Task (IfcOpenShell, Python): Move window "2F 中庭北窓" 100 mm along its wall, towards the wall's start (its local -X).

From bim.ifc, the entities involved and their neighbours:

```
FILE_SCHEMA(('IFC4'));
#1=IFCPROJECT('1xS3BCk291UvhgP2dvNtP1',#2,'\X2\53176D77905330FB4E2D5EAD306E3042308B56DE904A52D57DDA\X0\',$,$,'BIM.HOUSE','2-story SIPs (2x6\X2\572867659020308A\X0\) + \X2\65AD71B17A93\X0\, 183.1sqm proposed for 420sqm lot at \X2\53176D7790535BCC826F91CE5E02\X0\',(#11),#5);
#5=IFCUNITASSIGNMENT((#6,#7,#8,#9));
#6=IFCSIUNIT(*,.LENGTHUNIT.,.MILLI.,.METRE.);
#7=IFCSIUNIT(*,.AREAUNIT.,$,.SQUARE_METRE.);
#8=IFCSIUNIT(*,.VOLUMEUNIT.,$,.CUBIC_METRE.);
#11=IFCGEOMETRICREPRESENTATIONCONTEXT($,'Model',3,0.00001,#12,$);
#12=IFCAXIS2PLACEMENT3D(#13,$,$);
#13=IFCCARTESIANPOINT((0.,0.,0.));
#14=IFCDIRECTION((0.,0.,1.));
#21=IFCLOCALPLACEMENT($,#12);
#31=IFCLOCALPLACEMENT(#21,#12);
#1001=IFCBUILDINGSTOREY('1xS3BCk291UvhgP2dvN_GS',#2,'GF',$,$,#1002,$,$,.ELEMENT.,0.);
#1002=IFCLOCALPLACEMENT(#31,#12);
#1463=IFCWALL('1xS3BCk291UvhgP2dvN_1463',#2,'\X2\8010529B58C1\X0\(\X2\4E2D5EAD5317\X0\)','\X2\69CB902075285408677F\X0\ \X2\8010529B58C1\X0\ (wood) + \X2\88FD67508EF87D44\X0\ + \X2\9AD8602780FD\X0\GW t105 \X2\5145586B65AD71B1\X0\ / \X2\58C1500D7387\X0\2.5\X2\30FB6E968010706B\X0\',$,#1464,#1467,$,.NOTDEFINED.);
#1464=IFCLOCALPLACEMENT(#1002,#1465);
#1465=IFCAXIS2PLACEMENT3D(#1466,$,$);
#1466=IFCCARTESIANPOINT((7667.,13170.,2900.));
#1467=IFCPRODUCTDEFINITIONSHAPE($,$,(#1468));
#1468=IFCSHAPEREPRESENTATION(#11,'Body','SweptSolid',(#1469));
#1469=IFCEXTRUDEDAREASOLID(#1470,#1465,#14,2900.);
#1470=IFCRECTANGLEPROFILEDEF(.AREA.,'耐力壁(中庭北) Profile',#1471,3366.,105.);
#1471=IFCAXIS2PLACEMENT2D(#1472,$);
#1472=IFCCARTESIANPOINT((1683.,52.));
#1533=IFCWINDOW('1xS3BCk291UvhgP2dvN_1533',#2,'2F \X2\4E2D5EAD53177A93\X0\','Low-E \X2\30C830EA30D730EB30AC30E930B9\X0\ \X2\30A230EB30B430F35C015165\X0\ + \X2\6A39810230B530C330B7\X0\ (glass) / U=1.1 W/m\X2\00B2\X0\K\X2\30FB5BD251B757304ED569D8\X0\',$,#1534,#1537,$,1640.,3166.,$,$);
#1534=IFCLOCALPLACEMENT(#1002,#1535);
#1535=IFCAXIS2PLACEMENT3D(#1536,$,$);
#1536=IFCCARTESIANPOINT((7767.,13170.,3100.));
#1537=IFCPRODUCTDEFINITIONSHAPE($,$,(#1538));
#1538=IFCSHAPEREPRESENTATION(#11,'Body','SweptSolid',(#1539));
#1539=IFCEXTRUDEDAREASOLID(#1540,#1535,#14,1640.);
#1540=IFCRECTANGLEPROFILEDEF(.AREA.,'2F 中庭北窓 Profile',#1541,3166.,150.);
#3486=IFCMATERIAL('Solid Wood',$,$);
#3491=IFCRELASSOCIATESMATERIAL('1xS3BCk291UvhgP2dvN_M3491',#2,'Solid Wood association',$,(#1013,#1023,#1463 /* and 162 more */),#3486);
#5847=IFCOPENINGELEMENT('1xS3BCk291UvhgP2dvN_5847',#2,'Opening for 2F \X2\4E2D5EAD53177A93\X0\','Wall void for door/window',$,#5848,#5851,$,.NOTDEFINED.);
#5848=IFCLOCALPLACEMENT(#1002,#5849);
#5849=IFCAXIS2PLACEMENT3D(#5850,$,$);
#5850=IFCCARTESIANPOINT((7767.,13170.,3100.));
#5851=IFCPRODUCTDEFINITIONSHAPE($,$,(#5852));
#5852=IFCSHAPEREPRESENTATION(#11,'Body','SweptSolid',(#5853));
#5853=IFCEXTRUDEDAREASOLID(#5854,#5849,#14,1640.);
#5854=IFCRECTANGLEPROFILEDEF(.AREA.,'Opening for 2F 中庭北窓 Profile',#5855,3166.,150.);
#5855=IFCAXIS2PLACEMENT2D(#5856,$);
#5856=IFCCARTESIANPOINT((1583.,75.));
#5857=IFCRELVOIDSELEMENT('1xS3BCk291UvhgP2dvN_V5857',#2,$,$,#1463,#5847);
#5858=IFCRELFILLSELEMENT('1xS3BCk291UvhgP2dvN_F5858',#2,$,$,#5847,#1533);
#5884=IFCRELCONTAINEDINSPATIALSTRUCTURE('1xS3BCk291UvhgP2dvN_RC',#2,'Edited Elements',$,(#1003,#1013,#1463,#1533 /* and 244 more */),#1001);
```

```python
import ifcopenshell
import ifcopenshell.api.geometry
import ifcopenshell.util.placement
import ifcopenshell.util.unit

model = ifcopenshell.open("bim.ifc")
unit_scale = ifcopenshell.util.unit.calculate_unit_scale(model)

window = model.by_guid("1xS3BCk291UvhgP2dvN_1533")
opening = window.FillsVoids[0].RelatingOpeningElement
wall = opening.VoidsElements[0].RelatingBuildingElement

wall_matrix = ifcopenshell.util.placement.get_local_placement(wall.ObjectPlacement)
shift = wall_matrix[:3, 0] * -0.1 / unit_scale
before = ifcopenshell.util.placement.get_local_placement(window.ObjectPlacement)[:3, 3].copy()

# The window is not placed relative to its opening, so move both.
for product in (opening, window):
    matrix = ifcopenshell.util.placement.get_local_placement(product.ObjectPlacement)
    matrix[:3, 3] += shift
    ifcopenshell.api.geometry.edit_object_placement(model, product=product, matrix=matrix, is_si=False)

after = ifcopenshell.util.placement.get_local_placement(window.ObjectPlacement)[:3, 3]
print("window moved by", (after - before).round(3) + 0.0)

model.write("bim-out.ifc")
```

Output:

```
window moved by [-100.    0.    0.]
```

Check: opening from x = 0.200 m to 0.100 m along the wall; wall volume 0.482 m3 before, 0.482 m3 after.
